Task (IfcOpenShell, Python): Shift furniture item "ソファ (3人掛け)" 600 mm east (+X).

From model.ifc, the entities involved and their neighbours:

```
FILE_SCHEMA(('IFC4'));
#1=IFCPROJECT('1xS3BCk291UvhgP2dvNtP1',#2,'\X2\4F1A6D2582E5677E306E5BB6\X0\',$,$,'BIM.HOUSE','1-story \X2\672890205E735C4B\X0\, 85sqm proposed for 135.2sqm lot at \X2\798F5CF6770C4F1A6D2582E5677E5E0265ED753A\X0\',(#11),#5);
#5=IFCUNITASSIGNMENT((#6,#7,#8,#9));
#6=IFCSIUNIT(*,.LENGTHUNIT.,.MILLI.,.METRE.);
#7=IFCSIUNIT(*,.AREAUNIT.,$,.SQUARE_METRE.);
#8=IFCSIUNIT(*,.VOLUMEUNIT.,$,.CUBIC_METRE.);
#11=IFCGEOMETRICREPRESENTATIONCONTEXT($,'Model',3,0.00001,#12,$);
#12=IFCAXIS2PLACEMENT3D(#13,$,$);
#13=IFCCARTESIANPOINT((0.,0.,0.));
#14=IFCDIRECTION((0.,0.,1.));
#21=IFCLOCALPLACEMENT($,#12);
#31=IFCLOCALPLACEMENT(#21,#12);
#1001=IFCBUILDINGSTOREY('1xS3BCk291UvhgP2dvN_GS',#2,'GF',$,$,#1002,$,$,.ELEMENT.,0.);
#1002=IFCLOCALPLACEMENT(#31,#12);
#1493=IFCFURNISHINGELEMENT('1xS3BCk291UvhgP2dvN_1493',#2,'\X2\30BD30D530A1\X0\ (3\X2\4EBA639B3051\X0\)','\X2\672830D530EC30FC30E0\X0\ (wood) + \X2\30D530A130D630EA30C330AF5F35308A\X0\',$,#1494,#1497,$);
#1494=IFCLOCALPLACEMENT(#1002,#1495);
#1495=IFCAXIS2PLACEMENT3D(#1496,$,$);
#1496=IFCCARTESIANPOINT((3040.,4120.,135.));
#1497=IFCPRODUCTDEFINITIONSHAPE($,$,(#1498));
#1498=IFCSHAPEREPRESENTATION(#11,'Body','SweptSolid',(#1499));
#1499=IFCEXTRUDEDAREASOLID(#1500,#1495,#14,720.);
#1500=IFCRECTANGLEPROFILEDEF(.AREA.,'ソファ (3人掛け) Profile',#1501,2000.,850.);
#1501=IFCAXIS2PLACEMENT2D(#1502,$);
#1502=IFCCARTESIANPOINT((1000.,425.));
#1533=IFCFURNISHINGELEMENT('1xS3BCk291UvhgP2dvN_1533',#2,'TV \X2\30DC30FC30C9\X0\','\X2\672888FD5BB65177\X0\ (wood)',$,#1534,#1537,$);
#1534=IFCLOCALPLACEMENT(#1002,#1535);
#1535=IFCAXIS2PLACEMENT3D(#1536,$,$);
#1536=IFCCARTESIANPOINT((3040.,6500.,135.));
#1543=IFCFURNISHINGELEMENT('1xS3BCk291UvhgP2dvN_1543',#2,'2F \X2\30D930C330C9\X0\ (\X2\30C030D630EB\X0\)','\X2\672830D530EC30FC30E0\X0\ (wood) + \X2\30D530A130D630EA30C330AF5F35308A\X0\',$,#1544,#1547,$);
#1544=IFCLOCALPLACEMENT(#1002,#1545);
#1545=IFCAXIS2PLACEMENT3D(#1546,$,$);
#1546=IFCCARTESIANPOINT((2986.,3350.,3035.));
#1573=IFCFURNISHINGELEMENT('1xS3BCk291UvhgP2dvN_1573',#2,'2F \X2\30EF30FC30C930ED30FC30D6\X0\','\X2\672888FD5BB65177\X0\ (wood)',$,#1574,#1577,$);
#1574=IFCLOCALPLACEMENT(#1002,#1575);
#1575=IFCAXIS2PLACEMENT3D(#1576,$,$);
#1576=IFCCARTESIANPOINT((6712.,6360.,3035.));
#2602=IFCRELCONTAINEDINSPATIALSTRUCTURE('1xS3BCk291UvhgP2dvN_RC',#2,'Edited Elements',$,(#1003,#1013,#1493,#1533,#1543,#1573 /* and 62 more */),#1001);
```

```python
import ifcopenshell
import ifcopenshell.api.geometry
import ifcopenshell.util.placement
import ifcopenshell.util.unit

model = ifcopenshell.open("model.ifc")
unit_scale = ifcopenshell.util.unit.calculate_unit_scale(model)

item = model.by_guid("1xS3BCk291UvhgP2dvN_1493")
matrix = ifcopenshell.util.placement.get_local_placement(item.ObjectPlacement)
matrix[0, 3] += 0.6 / unit_scale
ifcopenshell.api.geometry.edit_object_placement(model, product=item, matrix=matrix, is_si=False)

print(ifcopenshell.util.placement.get_local_placement(item.ObjectPlacement).round(3) + 0.0)

model.write("model_edited.ifc")
```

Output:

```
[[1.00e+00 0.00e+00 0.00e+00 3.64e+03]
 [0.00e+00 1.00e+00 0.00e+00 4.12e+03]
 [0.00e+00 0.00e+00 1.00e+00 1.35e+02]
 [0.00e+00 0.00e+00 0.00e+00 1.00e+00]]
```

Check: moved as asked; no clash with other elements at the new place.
